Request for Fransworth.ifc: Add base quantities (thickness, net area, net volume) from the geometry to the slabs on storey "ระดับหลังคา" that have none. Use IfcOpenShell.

First a look at what the model holds.

```python
import ifcopenshell
import ifcopenshell.util.element
import ifcopenshell.util.unit

model = ifcopenshell.open("Fransworth.ifc")
print(model.schema)
for unit_type in ("LENGTHUNIT", "AREAUNIT", "VOLUMEUNIT"):
    print(unit_type, ifcopenshell.util.unit.calculate_unit_scale(model, unit_type))
storey = next(s for s in model.by_type("IfcBuildingStorey") if s.Name == "ระดับหลังคา")
slabs = [e for e in ifcopenshell.util.element.get_decomposition(storey) if e.is_a("IfcSlab")]
for e in sorted(slabs, key=lambda e: e.id()):
    print(e.id(), e.is_a(), e.Name, list(ifcopenshell.util.element.get_psets(e, qtos_only=True)), sep=" | ")
```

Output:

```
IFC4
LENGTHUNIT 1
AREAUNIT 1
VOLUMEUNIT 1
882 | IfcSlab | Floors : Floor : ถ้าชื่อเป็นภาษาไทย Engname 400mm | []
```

```python
import ifcopenshell
import ifcopenshell.api.pset
import ifcopenshell.geom
import ifcopenshell.util.element
import ifcopenshell.util.shape
import ifcopenshell.util.unit

model = ifcopenshell.open("Fransworth.ifc")
unit_scale = ifcopenshell.util.unit.calculate_unit_scale(model)
area_scale = ifcopenshell.util.unit.calculate_unit_scale(model, "AREAUNIT")
volume_scale = ifcopenshell.util.unit.calculate_unit_scale(model, "VOLUMEUNIT")
settings = ifcopenshell.geom.settings()

storey = next(s for s in model.by_type("IfcBuildingStorey") if s.Name == "ระดับหลังคา")
slabs = [e for e in ifcopenshell.util.element.get_decomposition(storey) if e.is_a("IfcSlab")]

for e in sorted(slabs, key=lambda e: e.id()):
    if ifcopenshell.util.element.get_psets(e, qtos_only=True, should_inherit=False):
        continue
    # Geometry comes back in metres, in the element's own axes.
    shape = ifcopenshell.geom.create_shape(settings, e)
    values = {
        "Width": ifcopenshell.util.shape.get_z(shape.geometry) / unit_scale,
        "NetArea": ifcopenshell.util.shape.get_footprint_area(shape.geometry) / area_scale,
        "NetVolume": ifcopenshell.util.shape.get_volume(shape.geometry) / volume_scale,
    }
    qto = ifcopenshell.api.pset.add_qto(model, product=e, name="Qto_SlabBaseQuantities")
    ifcopenshell.api.pset.edit_qto(model, qto=qto, properties=values)
    print(e.id(), {k: round(v, 3) for k, v in values.items()})

model.write("Fransworth-out.ifc")
```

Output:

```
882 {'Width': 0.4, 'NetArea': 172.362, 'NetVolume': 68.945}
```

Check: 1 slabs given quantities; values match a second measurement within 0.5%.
